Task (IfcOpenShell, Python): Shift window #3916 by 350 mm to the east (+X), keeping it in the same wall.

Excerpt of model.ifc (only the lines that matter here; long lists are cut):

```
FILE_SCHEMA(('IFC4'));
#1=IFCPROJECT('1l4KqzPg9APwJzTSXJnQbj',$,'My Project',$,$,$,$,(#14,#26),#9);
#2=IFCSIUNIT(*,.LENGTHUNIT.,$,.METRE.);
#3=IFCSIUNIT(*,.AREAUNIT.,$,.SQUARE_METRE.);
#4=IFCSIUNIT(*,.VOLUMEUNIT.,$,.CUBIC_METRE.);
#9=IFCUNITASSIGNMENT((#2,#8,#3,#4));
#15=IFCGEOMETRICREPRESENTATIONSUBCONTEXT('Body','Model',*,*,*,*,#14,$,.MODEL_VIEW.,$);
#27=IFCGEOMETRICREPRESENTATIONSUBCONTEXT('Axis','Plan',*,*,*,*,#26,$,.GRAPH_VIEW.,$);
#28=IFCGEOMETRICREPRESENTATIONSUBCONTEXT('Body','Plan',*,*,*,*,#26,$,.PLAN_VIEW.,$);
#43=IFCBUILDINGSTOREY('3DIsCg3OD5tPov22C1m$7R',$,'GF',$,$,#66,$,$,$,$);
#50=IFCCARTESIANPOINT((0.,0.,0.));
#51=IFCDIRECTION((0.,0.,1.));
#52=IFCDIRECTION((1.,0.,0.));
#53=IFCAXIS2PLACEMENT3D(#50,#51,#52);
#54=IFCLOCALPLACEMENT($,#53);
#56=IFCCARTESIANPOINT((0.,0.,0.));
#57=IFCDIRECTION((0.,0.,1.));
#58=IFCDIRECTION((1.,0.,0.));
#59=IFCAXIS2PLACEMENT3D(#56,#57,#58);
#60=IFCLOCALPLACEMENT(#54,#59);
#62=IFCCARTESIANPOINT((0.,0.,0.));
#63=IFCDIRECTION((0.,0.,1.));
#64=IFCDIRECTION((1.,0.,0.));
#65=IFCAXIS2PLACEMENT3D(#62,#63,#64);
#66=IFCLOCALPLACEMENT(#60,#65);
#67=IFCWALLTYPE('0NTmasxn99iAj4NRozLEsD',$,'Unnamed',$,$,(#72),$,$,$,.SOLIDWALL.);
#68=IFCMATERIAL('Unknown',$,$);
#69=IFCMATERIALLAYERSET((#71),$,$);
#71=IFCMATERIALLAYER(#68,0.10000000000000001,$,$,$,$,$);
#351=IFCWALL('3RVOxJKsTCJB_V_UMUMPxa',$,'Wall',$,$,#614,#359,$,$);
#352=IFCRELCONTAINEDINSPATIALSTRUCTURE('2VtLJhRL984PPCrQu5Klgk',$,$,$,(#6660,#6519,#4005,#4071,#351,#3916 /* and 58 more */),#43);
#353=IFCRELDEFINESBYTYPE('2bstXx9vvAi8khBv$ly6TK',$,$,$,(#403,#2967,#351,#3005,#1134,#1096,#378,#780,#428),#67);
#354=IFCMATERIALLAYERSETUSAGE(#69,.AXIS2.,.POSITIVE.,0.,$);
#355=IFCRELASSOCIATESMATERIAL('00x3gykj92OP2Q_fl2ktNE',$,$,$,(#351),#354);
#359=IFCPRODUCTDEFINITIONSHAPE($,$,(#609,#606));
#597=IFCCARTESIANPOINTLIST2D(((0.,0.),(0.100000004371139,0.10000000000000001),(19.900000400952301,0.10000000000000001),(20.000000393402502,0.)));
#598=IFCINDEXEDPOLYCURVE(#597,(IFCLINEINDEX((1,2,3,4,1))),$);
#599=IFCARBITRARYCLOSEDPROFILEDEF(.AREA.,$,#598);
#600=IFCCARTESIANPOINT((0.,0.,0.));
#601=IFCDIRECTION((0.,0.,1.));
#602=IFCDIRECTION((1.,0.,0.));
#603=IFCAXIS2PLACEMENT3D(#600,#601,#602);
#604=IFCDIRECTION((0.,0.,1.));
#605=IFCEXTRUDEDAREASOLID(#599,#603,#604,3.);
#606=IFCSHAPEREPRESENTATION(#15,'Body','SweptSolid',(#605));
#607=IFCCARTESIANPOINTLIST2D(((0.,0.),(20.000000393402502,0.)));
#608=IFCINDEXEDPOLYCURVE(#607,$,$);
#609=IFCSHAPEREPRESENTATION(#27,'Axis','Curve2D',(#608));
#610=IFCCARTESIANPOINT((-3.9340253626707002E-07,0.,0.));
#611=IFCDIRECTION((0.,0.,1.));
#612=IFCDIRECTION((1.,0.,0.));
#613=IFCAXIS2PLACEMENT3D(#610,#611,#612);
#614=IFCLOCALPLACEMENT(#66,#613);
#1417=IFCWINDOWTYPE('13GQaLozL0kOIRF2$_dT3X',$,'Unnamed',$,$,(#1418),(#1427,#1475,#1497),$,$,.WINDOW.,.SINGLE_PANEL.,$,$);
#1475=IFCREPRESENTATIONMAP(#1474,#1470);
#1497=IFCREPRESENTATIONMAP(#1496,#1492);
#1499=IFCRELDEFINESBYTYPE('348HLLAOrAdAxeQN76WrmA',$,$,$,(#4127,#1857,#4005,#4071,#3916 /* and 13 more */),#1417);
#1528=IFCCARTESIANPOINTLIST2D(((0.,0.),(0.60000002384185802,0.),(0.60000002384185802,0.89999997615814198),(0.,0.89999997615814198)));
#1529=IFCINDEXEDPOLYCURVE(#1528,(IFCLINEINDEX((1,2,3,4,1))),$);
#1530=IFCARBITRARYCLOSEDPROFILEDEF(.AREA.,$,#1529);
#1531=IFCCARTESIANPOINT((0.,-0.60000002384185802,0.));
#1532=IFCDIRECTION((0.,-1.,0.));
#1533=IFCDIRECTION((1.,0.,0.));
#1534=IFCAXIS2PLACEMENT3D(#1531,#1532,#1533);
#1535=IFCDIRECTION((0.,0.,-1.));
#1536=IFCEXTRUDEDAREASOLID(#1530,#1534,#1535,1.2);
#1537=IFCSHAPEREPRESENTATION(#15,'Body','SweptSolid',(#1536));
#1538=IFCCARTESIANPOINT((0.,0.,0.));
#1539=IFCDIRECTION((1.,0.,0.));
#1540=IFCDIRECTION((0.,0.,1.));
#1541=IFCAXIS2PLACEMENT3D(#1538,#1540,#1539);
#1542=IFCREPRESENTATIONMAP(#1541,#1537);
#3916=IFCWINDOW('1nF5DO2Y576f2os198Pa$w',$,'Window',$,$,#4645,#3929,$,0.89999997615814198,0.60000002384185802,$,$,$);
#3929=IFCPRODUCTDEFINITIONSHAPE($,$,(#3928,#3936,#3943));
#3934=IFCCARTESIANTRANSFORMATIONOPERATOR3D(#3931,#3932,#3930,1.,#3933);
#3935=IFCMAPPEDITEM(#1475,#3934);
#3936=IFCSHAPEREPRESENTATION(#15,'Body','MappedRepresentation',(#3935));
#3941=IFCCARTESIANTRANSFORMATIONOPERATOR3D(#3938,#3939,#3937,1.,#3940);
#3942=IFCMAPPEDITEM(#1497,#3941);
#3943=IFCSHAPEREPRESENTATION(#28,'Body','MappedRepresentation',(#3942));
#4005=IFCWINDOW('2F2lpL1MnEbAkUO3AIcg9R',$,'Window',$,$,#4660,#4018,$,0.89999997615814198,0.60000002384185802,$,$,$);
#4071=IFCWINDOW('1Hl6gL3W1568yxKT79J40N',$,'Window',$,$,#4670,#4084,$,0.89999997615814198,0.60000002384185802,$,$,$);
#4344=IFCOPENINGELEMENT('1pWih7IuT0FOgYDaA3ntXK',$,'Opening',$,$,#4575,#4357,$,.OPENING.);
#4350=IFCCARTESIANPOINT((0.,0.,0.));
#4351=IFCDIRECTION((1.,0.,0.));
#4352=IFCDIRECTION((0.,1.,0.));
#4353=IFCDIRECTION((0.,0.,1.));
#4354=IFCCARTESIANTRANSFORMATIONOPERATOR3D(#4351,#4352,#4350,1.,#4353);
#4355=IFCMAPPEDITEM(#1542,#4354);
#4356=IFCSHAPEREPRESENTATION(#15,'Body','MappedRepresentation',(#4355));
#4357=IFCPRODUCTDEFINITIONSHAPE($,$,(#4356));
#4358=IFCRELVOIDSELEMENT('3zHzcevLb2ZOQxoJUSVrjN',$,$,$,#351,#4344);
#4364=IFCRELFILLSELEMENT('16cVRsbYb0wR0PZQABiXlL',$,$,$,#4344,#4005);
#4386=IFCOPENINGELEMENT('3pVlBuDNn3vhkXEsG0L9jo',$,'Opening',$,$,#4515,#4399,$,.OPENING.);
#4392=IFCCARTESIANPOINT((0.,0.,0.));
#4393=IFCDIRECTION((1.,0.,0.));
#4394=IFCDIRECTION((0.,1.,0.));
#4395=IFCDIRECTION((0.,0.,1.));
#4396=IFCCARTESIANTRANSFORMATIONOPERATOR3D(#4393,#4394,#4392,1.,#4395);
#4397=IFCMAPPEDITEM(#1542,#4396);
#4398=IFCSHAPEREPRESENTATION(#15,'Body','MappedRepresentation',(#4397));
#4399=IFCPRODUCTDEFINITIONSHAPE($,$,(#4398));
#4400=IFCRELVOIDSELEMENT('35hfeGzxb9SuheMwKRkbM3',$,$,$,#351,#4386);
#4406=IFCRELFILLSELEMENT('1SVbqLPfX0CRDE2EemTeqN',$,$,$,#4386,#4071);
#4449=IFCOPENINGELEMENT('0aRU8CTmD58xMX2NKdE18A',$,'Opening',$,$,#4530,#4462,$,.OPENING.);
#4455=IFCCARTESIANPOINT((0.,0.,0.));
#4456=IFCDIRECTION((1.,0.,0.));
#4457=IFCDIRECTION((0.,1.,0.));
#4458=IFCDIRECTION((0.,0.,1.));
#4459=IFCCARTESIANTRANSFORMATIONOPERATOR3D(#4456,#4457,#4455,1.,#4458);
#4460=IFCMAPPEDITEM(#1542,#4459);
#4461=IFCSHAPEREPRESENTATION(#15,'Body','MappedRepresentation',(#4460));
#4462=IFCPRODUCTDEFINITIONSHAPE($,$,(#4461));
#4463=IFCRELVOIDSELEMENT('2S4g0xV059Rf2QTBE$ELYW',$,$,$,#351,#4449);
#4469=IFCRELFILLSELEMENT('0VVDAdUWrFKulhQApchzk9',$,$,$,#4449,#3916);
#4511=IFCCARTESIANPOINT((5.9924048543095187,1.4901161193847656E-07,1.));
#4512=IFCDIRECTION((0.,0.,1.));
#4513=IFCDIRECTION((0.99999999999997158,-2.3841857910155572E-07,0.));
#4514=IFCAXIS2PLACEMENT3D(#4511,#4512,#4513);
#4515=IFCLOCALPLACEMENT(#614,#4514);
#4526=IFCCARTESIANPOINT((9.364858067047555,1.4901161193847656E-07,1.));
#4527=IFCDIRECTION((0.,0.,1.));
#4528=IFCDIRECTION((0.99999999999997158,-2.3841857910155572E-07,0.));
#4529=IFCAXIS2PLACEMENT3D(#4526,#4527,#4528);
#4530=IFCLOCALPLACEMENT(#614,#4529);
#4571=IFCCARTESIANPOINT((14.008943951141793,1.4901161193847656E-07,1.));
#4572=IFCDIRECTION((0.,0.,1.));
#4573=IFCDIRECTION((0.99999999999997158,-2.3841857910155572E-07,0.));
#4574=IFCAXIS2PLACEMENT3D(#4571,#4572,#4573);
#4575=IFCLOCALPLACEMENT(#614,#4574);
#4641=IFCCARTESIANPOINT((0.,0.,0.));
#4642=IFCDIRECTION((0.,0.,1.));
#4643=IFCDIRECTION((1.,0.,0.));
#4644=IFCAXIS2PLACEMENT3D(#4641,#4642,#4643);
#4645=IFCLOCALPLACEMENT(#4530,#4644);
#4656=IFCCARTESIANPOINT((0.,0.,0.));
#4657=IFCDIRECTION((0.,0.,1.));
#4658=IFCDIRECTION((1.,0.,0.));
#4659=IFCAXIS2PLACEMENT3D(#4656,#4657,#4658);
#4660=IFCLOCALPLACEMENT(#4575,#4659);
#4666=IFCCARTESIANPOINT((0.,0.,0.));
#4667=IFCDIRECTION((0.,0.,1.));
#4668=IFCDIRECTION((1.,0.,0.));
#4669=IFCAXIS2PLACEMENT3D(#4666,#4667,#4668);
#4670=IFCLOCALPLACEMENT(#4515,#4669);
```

```python
import ifcopenshell
import ifcopenshell.api.geometry
import ifcopenshell.util.placement
import ifcopenshell.util.unit

model = ifcopenshell.open("model.ifc")
unit_scale = ifcopenshell.util.unit.calculate_unit_scale(model)

window = model.by_id(3916)
opening = window.FillsVoids[0].RelatingOpeningElement
wall = opening.VoidsElements[0].RelatingBuildingElement

wall_matrix = ifcopenshell.util.placement.get_local_placement(wall.ObjectPlacement)
shift = wall_matrix[:3, 0] * 0.35 / unit_scale
before = ifcopenshell.util.placement.get_local_placement(window.ObjectPlacement)[:3, 3].copy()

# The window is placed relative to its opening, so it follows when the opening moves.
matrix = ifcopenshell.util.placement.get_local_placement(opening.ObjectPlacement)
matrix[:3, 3] += shift
ifcopenshell.api.geometry.edit_object_placement(
    model, product=opening, matrix=matrix, is_si=False, should_transform_children=True
)

after = ifcopenshell.util.placement.get_local_placement(window.ObjectPlacement)[:3, 3]
print("window moved by", (after - before).round(3) + 0.0)

model.write("model_edited.ifc")
```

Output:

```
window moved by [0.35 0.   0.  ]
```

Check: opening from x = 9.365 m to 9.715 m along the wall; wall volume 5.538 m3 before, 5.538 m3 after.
